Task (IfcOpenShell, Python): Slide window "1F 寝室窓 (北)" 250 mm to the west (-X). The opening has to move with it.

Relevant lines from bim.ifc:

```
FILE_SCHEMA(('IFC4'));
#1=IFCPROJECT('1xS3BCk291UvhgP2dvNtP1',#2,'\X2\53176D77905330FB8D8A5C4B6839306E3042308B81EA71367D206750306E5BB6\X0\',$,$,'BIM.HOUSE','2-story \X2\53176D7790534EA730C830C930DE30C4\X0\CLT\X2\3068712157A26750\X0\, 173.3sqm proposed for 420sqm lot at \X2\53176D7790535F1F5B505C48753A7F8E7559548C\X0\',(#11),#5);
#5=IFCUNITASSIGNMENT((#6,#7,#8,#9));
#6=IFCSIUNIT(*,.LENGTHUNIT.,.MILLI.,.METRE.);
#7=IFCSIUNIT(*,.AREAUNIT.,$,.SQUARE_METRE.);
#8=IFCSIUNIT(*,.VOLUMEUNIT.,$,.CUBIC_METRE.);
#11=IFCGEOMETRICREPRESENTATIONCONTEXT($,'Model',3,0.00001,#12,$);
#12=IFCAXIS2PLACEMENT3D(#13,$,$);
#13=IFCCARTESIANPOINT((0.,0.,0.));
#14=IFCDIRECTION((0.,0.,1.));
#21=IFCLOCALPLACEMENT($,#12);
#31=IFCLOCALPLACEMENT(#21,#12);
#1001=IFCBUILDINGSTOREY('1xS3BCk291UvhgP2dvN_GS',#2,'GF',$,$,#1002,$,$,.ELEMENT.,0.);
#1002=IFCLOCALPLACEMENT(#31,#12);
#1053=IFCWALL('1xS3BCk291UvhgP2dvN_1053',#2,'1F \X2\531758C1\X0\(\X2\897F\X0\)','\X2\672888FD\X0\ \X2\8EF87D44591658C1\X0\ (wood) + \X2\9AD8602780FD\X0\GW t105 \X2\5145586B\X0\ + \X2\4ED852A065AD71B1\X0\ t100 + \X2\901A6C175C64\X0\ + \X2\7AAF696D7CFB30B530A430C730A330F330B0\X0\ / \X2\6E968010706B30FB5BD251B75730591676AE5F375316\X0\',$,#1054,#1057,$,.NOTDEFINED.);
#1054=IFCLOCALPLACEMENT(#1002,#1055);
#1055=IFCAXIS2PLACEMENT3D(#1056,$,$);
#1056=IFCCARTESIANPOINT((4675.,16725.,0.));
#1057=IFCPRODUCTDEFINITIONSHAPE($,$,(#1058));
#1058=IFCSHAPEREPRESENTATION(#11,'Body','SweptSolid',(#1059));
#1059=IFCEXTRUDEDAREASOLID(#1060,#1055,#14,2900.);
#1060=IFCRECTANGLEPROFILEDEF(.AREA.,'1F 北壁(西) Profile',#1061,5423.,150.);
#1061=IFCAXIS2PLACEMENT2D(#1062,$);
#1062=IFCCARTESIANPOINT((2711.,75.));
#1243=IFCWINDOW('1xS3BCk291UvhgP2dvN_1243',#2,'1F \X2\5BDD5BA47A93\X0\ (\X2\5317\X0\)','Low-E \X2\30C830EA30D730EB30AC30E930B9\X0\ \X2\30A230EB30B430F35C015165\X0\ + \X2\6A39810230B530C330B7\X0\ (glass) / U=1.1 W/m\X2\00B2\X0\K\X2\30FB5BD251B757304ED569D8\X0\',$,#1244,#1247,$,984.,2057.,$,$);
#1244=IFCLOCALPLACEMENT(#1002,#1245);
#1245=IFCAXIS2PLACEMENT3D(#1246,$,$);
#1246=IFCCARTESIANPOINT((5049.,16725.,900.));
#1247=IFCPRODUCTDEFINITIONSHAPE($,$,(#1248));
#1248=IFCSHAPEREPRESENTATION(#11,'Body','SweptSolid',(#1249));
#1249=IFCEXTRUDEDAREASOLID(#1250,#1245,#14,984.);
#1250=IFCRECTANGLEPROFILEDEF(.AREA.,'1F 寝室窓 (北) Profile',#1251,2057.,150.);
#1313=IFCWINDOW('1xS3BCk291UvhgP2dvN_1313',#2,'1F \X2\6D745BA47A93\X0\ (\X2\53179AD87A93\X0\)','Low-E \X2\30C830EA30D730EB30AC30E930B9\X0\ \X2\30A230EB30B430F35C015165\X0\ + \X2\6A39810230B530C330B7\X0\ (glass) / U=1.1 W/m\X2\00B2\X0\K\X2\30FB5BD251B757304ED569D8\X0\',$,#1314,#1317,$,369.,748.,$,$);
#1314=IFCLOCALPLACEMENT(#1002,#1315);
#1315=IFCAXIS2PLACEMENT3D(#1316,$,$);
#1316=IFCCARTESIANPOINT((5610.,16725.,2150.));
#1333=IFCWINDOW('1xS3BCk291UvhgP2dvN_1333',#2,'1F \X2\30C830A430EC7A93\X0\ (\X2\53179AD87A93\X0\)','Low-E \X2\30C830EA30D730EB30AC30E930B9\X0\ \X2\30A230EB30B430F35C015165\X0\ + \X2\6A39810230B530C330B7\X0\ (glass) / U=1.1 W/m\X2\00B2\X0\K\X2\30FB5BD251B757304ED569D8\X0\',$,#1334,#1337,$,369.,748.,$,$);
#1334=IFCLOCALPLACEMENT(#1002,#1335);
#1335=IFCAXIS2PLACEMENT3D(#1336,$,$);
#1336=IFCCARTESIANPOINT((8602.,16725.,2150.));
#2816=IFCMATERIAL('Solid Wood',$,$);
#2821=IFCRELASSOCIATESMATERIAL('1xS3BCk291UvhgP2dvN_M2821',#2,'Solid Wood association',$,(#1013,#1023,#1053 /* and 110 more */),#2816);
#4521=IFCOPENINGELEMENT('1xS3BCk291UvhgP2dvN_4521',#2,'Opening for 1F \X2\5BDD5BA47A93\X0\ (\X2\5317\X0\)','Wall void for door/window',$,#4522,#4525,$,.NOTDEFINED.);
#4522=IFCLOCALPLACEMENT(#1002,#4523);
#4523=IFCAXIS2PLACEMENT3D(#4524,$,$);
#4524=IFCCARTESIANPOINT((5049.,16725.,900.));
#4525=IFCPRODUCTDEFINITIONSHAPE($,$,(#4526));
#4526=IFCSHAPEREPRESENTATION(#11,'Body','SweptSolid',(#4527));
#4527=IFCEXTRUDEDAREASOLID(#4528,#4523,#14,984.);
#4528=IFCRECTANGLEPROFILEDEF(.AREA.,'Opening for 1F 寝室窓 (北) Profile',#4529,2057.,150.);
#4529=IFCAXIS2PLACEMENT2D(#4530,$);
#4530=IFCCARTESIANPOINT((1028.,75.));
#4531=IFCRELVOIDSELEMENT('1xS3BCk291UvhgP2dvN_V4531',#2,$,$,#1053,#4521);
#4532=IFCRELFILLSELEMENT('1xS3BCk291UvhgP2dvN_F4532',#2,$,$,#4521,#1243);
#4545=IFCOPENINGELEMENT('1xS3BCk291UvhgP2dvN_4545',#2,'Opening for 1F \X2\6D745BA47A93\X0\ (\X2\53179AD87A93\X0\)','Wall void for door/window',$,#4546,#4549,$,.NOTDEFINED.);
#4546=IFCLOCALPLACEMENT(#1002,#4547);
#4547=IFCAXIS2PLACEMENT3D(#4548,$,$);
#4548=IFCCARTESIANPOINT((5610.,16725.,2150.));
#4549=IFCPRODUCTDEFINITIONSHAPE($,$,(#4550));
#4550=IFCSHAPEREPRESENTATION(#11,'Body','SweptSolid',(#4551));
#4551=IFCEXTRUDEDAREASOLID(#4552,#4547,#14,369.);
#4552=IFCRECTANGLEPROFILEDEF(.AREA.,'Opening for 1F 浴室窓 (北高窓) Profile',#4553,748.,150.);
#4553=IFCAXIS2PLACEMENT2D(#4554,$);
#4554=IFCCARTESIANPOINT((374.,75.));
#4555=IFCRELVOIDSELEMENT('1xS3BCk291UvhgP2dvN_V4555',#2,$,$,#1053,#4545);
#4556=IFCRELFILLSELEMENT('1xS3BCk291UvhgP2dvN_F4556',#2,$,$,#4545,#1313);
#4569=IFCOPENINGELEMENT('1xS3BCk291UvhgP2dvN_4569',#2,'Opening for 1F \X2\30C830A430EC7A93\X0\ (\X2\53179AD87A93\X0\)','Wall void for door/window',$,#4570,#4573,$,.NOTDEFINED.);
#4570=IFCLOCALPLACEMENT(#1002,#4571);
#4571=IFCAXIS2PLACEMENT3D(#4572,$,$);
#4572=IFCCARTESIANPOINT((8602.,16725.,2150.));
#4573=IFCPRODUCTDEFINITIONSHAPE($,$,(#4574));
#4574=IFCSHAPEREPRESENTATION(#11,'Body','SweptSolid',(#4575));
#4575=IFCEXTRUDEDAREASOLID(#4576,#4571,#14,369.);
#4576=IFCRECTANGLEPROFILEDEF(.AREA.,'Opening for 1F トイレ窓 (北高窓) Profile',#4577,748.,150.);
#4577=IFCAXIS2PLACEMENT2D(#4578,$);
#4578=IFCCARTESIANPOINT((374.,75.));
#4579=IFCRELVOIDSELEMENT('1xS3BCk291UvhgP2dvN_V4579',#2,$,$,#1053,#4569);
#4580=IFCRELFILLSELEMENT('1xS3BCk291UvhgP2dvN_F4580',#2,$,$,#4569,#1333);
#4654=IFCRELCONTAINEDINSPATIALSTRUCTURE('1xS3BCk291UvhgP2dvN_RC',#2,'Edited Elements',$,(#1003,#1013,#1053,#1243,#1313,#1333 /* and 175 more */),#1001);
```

```python
import ifcopenshell
import ifcopenshell.api.geometry
import ifcopenshell.util.placement

model = ifcopenshell.open("bim.ifc")

window = model.by_id(1243)
opening = window.FillsVoids[0].RelatingOpeningElement
wall = opening.VoidsElements[0].RelatingBuildingElement

wall_matrix = ifcopenshell.util.placement.get_local_placement(wall.ObjectPlacement)
shift = wall_matrix[:3, 0] * -250.0
before = ifcopenshell.util.placement.get_local_placement(window.ObjectPlacement)[:3, 3].copy()

# The window is not placed relative to its opening, so move both.
for product in (opening, window):
    matrix = ifcopenshell.util.placement.get_local_placement(product.ObjectPlacement)
    matrix[:3, 3] += shift
    ifcopenshell.api.geometry.edit_object_placement(model, product=product, matrix=matrix, is_si=False)

after = ifcopenshell.util.placement.get_local_placement(window.ObjectPlacement)[:3, 3]
print("window moved by", (after - before).round(3) + 0.0)

model.write("bim_updated.ifc")
```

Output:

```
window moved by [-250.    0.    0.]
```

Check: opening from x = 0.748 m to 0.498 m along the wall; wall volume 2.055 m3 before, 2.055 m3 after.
